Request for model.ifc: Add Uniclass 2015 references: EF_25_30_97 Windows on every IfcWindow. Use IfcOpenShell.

First a look at what the model holds.

```python
import ifcopenshell

model = ifcopenshell.open("model.ifc")
print(model.schema)
print("classifications:", [c.Name for c in model.by_type("IfcClassification")])
for ifc_class in ("IfcDoor", "IfcRoof", "IfcStair", "IfcWall", "IfcWindow"):
    print(ifc_class, len(model.by_type(ifc_class)))
```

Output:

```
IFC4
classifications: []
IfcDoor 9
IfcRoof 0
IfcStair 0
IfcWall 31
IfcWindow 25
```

```python
import ifcopenshell
import ifcopenshell.api.classification

model = ifcopenshell.open("model.ifc")

system = ifcopenshell.api.classification.add_classification(model, classification="Uniclass 2015")

codes = {
    "IfcWindow": ("EF_25_30_97", "Windows"),
}
for ifc_class, (code, name) in codes.items():
    products = model.by_type(ifc_class)
    ifcopenshell.api.classification.add_reference(
        model, products=products, classification=system, identification=code, name=name
    )
    print(code, len(products))

model.write("model-out.ifc")
```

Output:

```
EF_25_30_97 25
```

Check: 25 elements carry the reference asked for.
